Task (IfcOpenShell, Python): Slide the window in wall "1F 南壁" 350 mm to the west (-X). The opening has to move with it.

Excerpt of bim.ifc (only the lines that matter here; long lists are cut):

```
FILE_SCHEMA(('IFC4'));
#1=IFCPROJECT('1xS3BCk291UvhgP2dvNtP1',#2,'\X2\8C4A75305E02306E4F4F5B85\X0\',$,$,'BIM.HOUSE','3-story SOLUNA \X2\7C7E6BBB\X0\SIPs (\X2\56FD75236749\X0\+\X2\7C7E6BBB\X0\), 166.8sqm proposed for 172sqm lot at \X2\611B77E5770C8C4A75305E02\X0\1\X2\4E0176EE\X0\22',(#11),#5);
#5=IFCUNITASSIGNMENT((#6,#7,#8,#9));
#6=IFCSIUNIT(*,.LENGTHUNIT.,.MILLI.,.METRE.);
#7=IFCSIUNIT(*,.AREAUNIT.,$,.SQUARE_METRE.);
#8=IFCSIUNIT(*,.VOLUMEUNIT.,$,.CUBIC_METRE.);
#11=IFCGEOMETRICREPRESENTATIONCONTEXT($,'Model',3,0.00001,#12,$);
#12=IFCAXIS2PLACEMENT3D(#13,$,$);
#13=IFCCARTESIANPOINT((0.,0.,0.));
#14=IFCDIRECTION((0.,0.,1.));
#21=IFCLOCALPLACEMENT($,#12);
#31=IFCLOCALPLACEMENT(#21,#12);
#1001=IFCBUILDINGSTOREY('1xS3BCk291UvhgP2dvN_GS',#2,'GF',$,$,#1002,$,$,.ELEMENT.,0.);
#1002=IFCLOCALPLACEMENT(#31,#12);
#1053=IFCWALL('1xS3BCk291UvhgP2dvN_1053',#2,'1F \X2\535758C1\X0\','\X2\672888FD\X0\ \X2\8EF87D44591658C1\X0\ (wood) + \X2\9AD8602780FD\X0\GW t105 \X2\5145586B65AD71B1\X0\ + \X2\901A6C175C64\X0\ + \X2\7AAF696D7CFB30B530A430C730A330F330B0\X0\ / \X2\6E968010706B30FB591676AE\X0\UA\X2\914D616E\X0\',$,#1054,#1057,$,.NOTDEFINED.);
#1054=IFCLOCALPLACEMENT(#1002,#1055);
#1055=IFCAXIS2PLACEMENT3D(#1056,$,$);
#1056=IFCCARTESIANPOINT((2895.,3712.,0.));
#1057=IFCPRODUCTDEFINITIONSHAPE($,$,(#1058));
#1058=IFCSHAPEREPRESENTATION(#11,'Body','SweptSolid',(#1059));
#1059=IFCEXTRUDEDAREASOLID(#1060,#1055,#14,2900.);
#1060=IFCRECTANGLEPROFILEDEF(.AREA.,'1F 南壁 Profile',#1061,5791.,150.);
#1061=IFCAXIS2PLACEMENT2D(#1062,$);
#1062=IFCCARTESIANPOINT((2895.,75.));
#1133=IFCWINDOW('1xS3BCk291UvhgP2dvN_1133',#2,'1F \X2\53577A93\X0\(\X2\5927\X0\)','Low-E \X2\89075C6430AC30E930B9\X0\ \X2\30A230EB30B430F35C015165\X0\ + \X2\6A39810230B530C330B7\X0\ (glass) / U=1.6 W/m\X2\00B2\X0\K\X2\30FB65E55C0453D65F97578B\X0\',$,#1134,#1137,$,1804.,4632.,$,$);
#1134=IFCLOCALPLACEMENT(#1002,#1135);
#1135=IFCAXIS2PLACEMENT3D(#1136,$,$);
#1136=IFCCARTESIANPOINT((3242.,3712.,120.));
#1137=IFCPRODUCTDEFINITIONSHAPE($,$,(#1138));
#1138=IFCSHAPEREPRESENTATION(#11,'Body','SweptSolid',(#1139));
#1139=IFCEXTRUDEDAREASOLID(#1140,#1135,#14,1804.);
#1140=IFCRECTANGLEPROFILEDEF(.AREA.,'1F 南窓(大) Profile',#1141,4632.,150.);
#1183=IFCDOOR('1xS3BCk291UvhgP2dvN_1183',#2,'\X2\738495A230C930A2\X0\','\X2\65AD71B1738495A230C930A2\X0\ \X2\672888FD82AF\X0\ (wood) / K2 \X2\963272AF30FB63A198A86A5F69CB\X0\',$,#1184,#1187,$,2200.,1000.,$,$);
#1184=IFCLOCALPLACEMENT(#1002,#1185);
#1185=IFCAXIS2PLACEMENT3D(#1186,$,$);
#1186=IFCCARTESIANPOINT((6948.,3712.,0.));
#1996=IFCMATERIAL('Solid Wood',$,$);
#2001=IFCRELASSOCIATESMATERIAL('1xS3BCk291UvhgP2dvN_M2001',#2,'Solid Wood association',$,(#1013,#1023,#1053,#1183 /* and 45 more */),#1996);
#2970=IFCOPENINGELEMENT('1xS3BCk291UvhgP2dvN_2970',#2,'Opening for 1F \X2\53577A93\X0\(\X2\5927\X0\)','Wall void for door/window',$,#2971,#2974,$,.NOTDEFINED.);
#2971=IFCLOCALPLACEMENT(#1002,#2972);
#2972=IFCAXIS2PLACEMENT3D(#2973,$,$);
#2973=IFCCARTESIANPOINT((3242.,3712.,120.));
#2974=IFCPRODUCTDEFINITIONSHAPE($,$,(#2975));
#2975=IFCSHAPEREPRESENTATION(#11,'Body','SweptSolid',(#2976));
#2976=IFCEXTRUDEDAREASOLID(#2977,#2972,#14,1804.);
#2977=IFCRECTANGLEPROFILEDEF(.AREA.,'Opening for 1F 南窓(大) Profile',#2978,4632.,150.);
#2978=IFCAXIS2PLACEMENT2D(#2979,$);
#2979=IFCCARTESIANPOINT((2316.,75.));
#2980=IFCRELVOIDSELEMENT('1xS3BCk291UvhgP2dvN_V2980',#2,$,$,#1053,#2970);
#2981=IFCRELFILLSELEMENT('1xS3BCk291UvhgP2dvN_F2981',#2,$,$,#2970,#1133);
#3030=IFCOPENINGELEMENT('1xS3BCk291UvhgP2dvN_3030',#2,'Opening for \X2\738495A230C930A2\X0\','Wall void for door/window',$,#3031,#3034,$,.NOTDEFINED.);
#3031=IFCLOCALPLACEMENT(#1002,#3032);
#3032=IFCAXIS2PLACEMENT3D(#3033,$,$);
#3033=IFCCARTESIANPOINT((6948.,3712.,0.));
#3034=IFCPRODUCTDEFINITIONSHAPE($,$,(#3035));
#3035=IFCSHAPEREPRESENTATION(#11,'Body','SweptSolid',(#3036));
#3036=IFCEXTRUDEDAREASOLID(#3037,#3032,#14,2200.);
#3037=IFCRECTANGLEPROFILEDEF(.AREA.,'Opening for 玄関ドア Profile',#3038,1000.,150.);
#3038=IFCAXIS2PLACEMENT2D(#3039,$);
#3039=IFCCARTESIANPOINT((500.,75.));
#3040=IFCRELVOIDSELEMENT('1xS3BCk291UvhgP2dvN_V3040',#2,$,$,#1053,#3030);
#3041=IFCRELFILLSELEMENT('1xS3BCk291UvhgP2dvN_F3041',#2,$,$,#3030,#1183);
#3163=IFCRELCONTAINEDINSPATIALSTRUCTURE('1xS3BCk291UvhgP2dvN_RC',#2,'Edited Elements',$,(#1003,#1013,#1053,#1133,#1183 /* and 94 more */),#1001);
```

```python
import ifcopenshell
import ifcopenshell.api.geometry
import ifcopenshell.util.placement
import ifcopenshell.util.unit

model = ifcopenshell.open("bim.ifc")
unit_scale = ifcopenshell.util.unit.calculate_unit_scale(model)

window = model.by_guid("1xS3BCk291UvhgP2dvN_1133")
opening = window.FillsVoids[0].RelatingOpeningElement
wall = opening.VoidsElements[0].RelatingBuildingElement

wall_matrix = ifcopenshell.util.placement.get_local_placement(wall.ObjectPlacement)
shift = wall_matrix[:3, 0] * -0.35 / unit_scale
before = ifcopenshell.util.placement.get_local_placement(window.ObjectPlacement)[:3, 3].copy()

# The window is not placed relative to its opening, so move both.
for product in (opening, window):
    matrix = ifcopenshell.util.placement.get_local_placement(product.ObjectPlacement)
    matrix[:3, 3] += shift
    ifcopenshell.api.geometry.edit_object_placement(model, product=product, matrix=matrix, is_si=False)

after = ifcopenshell.util.placement.get_local_placement(window.ObjectPlacement)[:3, 3]
print("window moved by", (after - before).round(3) + 0.0)

model.write("bim-out.ifc")
```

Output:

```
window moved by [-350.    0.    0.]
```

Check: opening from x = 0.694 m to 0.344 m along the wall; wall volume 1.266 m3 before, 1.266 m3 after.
